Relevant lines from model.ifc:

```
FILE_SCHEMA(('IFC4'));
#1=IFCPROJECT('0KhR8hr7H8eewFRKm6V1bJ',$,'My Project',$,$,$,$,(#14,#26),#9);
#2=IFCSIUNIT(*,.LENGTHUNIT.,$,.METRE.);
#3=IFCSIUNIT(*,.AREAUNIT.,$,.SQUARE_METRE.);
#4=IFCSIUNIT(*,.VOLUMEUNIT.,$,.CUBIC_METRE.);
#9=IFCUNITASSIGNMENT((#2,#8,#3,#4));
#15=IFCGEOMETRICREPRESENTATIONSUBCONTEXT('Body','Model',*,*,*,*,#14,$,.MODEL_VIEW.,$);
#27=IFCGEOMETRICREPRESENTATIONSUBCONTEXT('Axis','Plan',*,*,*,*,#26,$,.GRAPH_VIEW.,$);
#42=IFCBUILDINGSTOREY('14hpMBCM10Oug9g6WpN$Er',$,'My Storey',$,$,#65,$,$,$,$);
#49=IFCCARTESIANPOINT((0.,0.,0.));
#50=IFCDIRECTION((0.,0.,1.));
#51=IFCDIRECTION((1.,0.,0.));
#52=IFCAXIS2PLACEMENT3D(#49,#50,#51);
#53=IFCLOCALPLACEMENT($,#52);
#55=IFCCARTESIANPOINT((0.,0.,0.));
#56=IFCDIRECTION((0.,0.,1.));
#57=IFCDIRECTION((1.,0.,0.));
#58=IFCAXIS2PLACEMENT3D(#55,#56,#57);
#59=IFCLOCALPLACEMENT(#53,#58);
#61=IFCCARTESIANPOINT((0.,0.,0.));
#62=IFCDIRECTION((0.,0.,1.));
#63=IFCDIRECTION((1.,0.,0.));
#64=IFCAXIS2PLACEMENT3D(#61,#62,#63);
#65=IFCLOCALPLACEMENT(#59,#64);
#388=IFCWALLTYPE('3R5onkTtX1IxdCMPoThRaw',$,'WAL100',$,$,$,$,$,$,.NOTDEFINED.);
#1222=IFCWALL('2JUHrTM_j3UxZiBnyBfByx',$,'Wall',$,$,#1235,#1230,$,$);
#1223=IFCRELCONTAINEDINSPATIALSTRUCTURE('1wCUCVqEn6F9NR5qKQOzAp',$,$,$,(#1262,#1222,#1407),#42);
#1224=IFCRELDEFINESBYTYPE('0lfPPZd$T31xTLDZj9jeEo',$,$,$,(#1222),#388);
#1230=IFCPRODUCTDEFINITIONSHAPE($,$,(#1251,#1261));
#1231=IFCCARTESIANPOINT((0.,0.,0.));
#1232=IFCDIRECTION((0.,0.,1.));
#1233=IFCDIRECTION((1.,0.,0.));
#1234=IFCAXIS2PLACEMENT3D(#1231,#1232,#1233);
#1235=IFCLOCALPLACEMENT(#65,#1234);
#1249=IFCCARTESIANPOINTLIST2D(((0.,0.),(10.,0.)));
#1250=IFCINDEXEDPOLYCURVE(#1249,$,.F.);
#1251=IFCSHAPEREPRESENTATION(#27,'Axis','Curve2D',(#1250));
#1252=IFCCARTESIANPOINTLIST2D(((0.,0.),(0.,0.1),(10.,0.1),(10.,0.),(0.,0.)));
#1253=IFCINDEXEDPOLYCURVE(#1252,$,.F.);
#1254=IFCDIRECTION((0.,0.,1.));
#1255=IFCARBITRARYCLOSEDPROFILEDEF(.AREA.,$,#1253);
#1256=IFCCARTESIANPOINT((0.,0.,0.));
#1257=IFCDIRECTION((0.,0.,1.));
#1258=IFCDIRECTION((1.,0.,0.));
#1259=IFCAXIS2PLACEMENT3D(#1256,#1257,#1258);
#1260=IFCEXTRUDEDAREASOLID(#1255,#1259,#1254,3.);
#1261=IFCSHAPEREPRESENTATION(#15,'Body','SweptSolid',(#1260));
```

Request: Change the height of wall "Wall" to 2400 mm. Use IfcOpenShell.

```python
import ifcopenshell
import ifcopenshell.geom
import ifcopenshell.util.representation
import ifcopenshell.util.shape
import ifcopenshell.util.unit

model = ifcopenshell.open("model.ifc")
unit_scale = ifcopenshell.util.unit.calculate_unit_scale(model)
settings = ifcopenshell.geom.settings()


def volume(element):
    """Net volume in cubic metres, openings subtracted."""
    shape = ifcopenshell.geom.create_shape(settings, element)
    return ifcopenshell.util.shape.get_volume(shape.geometry)


wall = model.by_guid("2JUHrTM_j3UxZiBnyBfByx")
before = volume(wall)

body = ifcopenshell.util.representation.get_representation(wall, "Model", "Body")
solid = body.Items[0]
old_height = solid.Depth
solid.Depth = 2.4 / unit_scale
after = volume(wall)

print(f"height {old_height:g} -> {solid.Depth:g}, volume {before:.3f} -> {after:.3f} m3")

model.write("model-out.ifc")
```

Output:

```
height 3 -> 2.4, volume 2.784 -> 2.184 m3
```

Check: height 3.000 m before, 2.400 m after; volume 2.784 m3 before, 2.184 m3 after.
